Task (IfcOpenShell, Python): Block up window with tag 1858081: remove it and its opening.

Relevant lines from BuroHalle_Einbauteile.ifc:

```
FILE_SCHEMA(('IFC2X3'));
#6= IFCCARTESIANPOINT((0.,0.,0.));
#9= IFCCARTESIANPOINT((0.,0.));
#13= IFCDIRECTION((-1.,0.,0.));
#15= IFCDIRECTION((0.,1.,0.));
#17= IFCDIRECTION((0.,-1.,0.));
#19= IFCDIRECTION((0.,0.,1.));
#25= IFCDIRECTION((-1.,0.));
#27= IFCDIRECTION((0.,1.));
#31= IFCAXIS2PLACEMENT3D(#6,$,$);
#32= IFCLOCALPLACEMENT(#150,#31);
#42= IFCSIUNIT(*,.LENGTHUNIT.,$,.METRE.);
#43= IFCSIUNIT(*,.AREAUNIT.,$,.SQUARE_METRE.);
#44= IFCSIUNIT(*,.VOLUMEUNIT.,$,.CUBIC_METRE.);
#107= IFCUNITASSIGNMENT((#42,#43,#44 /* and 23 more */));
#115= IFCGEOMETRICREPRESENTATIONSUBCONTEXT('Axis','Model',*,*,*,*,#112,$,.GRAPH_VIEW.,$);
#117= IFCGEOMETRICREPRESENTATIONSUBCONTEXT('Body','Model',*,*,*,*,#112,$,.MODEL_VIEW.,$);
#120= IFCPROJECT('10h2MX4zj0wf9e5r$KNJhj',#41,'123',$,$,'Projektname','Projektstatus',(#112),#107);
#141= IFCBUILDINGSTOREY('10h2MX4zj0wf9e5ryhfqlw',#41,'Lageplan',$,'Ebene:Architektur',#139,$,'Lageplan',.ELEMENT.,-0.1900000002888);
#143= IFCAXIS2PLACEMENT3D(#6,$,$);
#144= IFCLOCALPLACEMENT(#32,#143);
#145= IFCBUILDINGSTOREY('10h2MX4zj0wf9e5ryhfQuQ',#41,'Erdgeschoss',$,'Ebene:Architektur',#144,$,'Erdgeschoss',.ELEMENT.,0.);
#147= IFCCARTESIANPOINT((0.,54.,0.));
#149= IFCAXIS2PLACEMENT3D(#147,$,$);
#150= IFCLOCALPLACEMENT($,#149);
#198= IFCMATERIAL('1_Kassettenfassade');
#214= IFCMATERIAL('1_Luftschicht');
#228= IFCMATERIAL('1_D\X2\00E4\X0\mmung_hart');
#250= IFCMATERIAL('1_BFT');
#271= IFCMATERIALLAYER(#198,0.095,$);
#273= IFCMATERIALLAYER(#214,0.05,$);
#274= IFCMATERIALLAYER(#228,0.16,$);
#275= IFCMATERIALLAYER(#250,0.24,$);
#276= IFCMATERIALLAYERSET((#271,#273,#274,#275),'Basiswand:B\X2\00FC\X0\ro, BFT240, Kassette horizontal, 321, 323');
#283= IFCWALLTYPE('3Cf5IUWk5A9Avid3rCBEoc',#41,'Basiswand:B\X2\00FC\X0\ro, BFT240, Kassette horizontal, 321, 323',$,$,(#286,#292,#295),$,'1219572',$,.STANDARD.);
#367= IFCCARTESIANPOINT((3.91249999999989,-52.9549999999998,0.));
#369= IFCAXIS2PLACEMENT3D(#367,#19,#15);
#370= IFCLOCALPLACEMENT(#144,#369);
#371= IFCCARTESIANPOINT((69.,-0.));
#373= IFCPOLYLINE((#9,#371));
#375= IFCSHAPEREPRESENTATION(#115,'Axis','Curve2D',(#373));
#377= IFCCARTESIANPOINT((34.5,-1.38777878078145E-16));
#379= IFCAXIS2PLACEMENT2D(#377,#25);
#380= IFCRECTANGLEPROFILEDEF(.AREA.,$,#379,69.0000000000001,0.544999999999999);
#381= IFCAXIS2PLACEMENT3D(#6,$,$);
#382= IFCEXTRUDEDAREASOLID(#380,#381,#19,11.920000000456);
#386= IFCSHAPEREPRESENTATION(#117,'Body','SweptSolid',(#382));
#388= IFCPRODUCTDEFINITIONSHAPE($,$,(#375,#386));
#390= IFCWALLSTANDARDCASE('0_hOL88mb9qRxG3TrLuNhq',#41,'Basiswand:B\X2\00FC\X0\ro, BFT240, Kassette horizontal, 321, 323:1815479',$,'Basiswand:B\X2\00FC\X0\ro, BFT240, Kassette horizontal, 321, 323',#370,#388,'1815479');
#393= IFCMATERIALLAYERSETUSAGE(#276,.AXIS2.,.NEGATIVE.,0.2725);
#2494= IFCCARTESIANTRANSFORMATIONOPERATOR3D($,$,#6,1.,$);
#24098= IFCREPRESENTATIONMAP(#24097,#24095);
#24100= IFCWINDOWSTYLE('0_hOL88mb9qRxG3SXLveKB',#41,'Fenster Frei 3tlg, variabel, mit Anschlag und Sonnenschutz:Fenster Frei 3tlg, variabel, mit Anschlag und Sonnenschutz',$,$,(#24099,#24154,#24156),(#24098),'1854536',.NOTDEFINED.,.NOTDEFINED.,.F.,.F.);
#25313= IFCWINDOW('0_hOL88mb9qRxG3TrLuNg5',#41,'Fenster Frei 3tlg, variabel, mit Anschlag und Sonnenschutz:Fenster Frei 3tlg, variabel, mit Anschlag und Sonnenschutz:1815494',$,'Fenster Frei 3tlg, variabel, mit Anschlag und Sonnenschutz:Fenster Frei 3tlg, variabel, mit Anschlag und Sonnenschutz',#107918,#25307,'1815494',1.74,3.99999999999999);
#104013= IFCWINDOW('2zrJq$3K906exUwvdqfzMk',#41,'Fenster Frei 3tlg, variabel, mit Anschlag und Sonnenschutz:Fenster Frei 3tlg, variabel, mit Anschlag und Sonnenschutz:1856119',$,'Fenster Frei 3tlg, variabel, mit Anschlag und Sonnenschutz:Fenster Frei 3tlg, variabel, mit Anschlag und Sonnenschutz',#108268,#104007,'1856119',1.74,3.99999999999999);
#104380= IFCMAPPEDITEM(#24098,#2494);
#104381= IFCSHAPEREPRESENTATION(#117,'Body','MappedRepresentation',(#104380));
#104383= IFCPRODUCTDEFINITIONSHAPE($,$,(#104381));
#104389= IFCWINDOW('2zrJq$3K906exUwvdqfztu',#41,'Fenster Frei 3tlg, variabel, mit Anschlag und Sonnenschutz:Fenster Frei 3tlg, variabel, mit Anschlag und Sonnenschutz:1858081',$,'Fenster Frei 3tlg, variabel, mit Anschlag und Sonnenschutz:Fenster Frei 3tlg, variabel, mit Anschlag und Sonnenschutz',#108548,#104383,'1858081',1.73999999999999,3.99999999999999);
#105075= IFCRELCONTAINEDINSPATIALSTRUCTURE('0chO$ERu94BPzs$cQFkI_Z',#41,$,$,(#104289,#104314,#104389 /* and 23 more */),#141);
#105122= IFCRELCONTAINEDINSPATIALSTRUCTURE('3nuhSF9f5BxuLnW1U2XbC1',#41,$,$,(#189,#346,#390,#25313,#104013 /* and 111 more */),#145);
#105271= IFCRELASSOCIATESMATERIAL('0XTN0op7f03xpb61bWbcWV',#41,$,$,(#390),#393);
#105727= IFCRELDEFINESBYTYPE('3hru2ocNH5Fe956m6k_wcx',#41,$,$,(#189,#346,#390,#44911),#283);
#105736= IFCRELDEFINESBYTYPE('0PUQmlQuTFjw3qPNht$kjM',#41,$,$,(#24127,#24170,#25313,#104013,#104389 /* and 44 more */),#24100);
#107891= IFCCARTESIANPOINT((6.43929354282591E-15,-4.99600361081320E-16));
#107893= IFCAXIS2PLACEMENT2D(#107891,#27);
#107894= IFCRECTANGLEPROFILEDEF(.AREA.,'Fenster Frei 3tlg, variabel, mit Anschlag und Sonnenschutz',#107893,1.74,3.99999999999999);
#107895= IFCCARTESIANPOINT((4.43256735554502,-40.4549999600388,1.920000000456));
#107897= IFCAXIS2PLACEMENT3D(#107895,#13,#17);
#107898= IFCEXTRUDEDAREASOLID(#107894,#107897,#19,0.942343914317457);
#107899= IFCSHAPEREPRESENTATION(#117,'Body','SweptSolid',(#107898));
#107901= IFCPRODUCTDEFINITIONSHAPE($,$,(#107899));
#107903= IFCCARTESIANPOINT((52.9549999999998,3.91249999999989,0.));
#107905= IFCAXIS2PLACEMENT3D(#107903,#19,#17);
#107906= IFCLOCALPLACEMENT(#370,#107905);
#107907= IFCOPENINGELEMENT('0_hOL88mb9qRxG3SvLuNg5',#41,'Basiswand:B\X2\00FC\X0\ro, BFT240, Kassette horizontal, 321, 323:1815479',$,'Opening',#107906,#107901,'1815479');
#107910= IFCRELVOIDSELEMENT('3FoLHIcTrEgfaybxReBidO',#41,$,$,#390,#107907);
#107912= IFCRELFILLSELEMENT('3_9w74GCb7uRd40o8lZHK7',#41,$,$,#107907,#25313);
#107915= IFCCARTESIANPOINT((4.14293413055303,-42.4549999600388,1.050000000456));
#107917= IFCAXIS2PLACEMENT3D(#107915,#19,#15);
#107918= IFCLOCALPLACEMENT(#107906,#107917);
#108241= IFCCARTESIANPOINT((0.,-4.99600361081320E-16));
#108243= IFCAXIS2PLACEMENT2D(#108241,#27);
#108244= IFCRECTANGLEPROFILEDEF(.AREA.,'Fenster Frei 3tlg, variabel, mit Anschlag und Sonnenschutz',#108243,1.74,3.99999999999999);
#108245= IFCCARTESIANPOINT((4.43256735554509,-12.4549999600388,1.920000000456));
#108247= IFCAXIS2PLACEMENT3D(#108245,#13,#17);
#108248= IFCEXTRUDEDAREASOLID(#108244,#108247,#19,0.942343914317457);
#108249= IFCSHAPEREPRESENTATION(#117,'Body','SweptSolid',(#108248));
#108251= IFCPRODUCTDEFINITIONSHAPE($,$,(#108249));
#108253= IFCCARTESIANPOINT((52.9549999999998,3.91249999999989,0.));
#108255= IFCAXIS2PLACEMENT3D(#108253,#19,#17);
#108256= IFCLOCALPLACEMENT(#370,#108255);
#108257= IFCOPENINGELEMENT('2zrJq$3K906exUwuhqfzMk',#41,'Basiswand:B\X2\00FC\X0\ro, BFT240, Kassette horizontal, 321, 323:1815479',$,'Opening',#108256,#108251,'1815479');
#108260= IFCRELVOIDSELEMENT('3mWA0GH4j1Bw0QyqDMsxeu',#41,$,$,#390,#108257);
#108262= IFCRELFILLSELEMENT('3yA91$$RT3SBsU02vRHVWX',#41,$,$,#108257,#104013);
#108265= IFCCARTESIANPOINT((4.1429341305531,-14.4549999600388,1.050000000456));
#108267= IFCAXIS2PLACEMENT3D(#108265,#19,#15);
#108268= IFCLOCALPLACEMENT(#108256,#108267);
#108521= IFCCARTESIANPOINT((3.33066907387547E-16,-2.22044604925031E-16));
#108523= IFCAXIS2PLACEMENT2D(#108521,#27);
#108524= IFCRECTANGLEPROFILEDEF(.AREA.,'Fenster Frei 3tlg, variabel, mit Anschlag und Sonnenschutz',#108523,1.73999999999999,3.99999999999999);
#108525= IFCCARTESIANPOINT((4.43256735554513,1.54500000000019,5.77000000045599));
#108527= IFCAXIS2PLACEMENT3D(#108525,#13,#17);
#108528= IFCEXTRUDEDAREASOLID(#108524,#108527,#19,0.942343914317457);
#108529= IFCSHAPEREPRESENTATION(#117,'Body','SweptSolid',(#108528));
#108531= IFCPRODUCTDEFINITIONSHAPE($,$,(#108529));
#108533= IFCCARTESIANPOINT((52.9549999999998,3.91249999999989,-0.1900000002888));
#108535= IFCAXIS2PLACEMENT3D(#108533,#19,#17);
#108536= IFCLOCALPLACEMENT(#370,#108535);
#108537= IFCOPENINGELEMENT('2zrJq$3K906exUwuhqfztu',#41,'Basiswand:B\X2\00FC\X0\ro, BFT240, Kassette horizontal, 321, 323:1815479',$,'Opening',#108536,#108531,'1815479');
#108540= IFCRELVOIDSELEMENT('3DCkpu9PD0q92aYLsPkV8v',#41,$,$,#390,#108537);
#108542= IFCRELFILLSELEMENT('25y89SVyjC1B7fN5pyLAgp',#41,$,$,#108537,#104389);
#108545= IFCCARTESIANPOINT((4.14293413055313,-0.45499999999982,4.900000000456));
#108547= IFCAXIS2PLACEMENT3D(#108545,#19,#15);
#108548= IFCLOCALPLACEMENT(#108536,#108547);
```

```python
import ifcopenshell
import ifcopenshell.api.feature
import ifcopenshell.api.root
import ifcopenshell.geom
import ifcopenshell.util.shape

model = ifcopenshell.open("BuroHalle_Einbauteile.ifc")
settings = ifcopenshell.geom.settings()


def volume(element):
    """Net volume in cubic metres, openings subtracted."""
    shape = ifcopenshell.geom.create_shape(settings, element)
    return ifcopenshell.util.shape.get_volume(shape.geometry)


window = model.by_id(104389)
opening = window.FillsVoids[0].RelatingOpeningElement
wall = opening.VoidsElements[0].RelatingBuildingElement
before = volume(wall)

ifcopenshell.api.root.remove_product(model, product=window)
ifcopenshell.api.feature.remove_feature(model, feature=opening)

after = volume(wall)

print(f"wall volume {before:.3f} -> {after:.3f} m3")

model.write("BuroHalle_Einbauteile_rev.ifc")
```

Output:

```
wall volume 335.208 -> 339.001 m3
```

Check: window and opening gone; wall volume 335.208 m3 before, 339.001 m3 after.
